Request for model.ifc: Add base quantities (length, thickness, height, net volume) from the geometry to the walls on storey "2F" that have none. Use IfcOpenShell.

First a look at what the model holds.

```python
import ifcopenshell
import ifcopenshell.util.element
import ifcopenshell.util.unit

model = ifcopenshell.open("model.ifc")
print(model.schema)
for unit_type in ("LENGTHUNIT", "AREAUNIT", "VOLUMEUNIT"):
    print(unit_type, ifcopenshell.util.unit.calculate_unit_scale(model, unit_type))
storey = next(s for s in model.by_type("IfcBuildingStorey") if s.Name == "2F")
walls = [e for e in ifcopenshell.util.element.get_decomposition(storey) if e.is_a("IfcWall")]
for e in sorted(walls, key=lambda e: e.id()):
    print(e.id(), e.is_a(), e.Name, list(ifcopenshell.util.element.get_psets(e, qtos_only=True)), sep=" | ")
```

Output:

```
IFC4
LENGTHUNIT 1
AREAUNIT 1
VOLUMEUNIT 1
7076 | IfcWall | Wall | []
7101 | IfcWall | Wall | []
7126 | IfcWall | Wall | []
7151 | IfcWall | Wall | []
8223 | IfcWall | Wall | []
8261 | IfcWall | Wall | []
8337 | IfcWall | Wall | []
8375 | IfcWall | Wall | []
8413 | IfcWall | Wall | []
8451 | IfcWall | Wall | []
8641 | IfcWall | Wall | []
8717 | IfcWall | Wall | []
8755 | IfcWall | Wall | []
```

```python
import ifcopenshell
import ifcopenshell.api.pset
import ifcopenshell.geom
import ifcopenshell.util.element
import ifcopenshell.util.shape
import ifcopenshell.util.unit

model = ifcopenshell.open("model.ifc")
unit_scale = ifcopenshell.util.unit.calculate_unit_scale(model)
volume_scale = ifcopenshell.util.unit.calculate_unit_scale(model, "VOLUMEUNIT")
settings = ifcopenshell.geom.settings()

storey = next(s for s in model.by_type("IfcBuildingStorey") if s.Name == "2F")
walls = [e for e in ifcopenshell.util.element.get_decomposition(storey) if e.is_a("IfcWall")]

for e in sorted(walls, key=lambda e: e.id()):
    if ifcopenshell.util.element.get_psets(e, qtos_only=True, should_inherit=False):
        continue
    # Geometry comes back in metres, in the element's own axes.
    shape = ifcopenshell.geom.create_shape(settings, e)
    values = {
        "Length": ifcopenshell.util.shape.get_x(shape.geometry) / unit_scale,
        "Width": ifcopenshell.util.shape.get_y(shape.geometry) / unit_scale,
        "Height": ifcopenshell.util.shape.get_z(shape.geometry) / unit_scale,
        "NetVolume": ifcopenshell.util.shape.get_volume(shape.geometry) / volume_scale,
    }
    qto = ifcopenshell.api.pset.add_qto(model, product=e, name="Qto_WallBaseQuantities")
    ifcopenshell.api.pset.edit_qto(model, qto=qto, properties=values)
    print(e.id(), {k: round(v, 3) for k, v in values.items()})

model.write("model_edited.ifc")
```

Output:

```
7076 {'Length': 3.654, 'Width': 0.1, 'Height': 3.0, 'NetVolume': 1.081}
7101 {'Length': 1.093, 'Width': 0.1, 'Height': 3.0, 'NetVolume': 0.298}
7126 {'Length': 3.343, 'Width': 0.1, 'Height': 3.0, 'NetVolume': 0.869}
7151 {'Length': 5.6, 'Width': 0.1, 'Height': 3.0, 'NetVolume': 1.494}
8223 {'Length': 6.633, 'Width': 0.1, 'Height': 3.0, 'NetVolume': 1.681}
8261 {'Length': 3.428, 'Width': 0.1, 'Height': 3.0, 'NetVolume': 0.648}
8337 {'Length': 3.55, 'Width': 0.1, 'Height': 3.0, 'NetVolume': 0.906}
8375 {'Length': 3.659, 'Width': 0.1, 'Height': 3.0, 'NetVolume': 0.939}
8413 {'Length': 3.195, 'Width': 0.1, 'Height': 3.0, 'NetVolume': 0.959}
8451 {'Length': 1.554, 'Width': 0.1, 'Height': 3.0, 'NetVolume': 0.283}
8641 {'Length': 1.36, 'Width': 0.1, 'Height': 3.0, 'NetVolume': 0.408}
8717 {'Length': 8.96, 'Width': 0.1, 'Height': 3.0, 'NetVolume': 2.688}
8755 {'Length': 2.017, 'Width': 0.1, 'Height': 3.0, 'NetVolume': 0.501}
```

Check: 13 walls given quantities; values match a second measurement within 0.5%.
